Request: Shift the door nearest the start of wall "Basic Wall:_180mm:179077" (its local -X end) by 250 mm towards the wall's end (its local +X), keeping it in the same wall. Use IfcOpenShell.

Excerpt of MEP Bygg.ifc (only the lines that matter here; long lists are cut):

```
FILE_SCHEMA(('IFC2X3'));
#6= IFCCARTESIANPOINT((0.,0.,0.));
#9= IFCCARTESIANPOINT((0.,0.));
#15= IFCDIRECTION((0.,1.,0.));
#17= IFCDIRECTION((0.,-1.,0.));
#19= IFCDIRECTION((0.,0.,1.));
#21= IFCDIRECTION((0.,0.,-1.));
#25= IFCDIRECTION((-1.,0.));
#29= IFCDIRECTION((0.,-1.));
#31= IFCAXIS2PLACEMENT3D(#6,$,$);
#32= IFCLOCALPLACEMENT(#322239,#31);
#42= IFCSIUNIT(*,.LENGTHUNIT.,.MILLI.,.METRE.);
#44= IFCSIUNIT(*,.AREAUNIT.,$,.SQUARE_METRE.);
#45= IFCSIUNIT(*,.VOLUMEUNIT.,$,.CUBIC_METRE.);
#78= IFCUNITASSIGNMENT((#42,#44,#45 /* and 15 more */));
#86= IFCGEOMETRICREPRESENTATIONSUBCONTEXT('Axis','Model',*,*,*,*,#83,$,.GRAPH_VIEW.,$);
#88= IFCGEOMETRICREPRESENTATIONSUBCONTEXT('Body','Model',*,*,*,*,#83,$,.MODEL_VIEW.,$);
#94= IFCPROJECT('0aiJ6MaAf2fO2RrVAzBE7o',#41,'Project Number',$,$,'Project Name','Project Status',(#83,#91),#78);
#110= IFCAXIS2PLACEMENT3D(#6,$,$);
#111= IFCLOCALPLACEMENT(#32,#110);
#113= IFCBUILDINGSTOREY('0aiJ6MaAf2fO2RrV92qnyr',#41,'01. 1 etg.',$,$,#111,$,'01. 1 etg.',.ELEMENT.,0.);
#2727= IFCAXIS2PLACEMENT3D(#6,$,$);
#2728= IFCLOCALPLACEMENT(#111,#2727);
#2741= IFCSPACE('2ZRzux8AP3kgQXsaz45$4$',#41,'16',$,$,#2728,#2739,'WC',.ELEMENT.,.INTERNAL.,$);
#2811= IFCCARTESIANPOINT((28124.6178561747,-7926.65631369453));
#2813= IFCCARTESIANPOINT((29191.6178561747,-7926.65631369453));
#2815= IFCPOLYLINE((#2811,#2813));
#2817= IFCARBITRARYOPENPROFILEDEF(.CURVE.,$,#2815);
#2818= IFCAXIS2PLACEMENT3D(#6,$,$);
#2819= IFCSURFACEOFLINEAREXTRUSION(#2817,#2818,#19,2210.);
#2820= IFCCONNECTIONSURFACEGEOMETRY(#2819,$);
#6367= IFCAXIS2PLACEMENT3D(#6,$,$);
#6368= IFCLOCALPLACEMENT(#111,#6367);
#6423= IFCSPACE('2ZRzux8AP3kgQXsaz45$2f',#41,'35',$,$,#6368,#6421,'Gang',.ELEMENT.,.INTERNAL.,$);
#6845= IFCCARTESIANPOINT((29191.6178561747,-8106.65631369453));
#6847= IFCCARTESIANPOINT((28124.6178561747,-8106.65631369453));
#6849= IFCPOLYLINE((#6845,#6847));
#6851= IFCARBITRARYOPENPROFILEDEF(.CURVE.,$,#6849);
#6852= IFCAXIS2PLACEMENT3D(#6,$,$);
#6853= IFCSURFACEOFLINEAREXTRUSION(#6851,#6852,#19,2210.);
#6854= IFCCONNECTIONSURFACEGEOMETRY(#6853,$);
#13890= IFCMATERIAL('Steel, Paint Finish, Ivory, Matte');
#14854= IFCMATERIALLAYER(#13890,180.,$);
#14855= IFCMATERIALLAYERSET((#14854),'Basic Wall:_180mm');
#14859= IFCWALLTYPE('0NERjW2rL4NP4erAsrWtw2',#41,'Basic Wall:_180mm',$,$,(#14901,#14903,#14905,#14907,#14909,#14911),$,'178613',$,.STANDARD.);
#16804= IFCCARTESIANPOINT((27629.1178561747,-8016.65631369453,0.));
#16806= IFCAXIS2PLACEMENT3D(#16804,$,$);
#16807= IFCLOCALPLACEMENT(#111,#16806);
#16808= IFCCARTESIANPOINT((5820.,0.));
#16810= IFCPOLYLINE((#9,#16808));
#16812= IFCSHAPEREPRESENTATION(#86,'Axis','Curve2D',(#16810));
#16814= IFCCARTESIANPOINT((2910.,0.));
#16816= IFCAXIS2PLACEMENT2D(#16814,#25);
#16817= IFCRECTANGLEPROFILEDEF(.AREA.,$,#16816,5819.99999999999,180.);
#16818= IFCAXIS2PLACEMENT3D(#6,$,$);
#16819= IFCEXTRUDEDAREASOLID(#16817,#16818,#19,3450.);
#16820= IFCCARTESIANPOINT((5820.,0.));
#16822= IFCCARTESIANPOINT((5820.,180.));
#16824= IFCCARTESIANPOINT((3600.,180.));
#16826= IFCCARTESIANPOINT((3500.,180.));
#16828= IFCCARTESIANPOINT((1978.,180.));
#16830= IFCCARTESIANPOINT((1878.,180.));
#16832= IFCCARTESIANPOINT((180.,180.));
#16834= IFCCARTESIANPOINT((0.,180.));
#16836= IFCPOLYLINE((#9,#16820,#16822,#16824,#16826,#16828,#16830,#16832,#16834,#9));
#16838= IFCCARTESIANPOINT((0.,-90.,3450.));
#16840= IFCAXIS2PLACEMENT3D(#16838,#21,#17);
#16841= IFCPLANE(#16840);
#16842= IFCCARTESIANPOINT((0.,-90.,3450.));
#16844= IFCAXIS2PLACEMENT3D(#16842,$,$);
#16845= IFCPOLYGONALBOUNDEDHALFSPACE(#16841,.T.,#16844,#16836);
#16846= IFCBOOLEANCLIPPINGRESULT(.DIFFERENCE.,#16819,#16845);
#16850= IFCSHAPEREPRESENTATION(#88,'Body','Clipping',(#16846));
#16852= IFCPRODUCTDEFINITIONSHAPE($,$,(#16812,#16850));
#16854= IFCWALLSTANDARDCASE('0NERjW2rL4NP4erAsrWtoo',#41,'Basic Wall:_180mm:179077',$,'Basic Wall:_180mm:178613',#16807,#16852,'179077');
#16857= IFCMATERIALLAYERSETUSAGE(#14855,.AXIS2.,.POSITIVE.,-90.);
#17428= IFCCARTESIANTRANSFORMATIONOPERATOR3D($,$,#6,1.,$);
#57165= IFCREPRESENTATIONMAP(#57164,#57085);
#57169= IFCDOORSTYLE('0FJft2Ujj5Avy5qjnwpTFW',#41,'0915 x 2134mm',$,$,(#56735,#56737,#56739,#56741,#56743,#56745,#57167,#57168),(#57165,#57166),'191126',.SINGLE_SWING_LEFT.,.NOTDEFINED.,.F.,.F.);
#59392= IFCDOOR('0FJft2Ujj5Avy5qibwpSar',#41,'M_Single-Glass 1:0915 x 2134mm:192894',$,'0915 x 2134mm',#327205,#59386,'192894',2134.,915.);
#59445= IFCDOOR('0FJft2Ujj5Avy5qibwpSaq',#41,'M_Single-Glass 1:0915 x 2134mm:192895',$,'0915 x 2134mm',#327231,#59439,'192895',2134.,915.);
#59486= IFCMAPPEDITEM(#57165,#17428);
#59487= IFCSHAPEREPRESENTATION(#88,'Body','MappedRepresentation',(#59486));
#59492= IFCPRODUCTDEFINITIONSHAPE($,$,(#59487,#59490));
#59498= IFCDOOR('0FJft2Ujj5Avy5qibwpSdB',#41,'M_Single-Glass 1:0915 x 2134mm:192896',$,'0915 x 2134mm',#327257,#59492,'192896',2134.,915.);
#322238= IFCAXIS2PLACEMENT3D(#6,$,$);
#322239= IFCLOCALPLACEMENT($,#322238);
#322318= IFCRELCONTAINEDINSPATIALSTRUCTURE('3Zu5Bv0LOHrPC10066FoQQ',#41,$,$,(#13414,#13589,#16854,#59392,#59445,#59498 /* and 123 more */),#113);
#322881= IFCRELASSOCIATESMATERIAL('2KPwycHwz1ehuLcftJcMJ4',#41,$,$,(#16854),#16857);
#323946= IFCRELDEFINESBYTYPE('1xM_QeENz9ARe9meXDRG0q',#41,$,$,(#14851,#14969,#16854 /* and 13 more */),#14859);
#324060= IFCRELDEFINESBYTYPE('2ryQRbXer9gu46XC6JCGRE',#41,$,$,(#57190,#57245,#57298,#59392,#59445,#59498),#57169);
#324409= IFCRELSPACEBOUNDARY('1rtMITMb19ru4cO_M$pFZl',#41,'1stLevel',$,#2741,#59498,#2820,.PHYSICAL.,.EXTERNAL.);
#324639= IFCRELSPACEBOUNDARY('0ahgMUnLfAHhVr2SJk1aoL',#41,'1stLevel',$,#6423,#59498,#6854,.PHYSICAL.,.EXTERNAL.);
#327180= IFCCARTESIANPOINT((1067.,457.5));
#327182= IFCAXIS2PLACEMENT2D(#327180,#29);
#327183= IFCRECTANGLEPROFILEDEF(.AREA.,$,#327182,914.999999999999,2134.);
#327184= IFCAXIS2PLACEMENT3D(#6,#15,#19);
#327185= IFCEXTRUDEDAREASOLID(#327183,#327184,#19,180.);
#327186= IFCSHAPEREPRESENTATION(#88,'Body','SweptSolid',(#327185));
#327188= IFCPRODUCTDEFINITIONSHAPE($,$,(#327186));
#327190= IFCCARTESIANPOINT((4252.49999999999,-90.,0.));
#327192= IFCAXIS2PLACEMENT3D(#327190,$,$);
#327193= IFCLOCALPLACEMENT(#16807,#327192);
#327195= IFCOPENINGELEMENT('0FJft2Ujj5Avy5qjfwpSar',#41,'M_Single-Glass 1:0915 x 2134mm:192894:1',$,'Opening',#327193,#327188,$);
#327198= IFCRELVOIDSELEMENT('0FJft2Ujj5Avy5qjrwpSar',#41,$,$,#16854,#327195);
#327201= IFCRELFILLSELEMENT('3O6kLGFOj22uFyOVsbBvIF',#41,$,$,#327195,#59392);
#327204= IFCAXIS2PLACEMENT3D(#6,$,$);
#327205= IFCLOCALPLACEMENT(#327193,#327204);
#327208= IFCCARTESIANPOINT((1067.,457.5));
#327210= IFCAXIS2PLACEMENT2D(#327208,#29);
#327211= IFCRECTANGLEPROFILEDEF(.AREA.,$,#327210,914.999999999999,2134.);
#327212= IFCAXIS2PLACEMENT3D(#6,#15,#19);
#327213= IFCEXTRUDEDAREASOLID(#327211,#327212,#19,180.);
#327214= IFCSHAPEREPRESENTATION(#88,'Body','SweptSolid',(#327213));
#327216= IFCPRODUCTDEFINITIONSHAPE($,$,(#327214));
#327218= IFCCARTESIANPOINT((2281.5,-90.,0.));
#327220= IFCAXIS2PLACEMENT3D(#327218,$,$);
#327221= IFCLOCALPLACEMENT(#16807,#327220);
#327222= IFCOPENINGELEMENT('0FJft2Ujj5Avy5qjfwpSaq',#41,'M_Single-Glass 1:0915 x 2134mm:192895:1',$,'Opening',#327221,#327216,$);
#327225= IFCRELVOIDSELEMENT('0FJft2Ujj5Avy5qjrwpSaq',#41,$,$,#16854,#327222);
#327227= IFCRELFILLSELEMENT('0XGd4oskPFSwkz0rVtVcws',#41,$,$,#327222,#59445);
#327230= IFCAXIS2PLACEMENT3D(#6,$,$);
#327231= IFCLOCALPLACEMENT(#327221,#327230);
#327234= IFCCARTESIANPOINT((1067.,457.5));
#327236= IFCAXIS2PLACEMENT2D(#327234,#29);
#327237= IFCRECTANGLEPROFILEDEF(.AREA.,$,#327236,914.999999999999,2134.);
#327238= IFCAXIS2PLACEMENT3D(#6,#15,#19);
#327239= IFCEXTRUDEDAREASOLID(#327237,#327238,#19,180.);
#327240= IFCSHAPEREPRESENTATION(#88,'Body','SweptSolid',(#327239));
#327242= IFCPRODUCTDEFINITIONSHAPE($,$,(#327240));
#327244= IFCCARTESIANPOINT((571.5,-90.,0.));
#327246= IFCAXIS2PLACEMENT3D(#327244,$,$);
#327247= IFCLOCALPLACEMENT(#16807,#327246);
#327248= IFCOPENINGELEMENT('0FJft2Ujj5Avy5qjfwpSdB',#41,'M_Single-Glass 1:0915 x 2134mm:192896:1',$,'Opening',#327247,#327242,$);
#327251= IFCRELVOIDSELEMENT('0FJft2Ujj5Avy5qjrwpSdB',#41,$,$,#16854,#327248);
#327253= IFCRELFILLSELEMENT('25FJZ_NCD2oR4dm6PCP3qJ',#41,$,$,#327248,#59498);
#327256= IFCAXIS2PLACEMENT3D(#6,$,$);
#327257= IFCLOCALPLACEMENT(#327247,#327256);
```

```python
import numpy as np
import ifcopenshell
import ifcopenshell.api.geometry
import ifcopenshell.util.placement

model = ifcopenshell.open("MEP Bygg.ifc")

door = model.by_guid("0FJft2Ujj5Avy5qibwpSdB")
opening = door.FillsVoids[0].RelatingOpeningElement
wall = opening.VoidsElements[0].RelatingBuildingElement

wall_matrix = ifcopenshell.util.placement.get_local_placement(wall.ObjectPlacement)
shift = wall_matrix[:3, 0] * 250.0
before = ifcopenshell.util.placement.get_local_placement(door.ObjectPlacement)[:3, 3].copy()

# The door is placed relative to its opening, so it follows when the opening moves.
matrix = ifcopenshell.util.placement.get_local_placement(opening.ObjectPlacement)
matrix[:3, 3] += shift
ifcopenshell.api.geometry.edit_object_placement(
    model, product=opening, matrix=matrix, is_si=False, should_transform_children=True
)

# Space boundary surfaces are stored in each space's coordinates; move them too.
for rel in door.ProvidesBoundaries:
    if not rel.ConnectionGeometry:
        continue
    surface = rel.ConnectionGeometry.SurfaceOnRelatingElement
    space_matrix = ifcopenshell.util.placement.get_local_placement(rel.RelatingSpace.ObjectPlacement)
    point = np.array(surface.Position.Location.Coordinates) + space_matrix[:3, :3].T @ shift
    surface.Position = model.createIfcAxis2Placement3D(
        model.createIfcCartesianPoint(point.tolist()), surface.Position.Axis, surface.Position.RefDirection
    )

after = ifcopenshell.util.placement.get_local_placement(door.ObjectPlacement)[:3, 3]
print("door moved by", (after - before).round(3) + 0.0)

model.write("MEP Bygg_updated.ifc")
```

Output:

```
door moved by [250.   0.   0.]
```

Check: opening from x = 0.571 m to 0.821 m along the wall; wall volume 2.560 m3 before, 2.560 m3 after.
